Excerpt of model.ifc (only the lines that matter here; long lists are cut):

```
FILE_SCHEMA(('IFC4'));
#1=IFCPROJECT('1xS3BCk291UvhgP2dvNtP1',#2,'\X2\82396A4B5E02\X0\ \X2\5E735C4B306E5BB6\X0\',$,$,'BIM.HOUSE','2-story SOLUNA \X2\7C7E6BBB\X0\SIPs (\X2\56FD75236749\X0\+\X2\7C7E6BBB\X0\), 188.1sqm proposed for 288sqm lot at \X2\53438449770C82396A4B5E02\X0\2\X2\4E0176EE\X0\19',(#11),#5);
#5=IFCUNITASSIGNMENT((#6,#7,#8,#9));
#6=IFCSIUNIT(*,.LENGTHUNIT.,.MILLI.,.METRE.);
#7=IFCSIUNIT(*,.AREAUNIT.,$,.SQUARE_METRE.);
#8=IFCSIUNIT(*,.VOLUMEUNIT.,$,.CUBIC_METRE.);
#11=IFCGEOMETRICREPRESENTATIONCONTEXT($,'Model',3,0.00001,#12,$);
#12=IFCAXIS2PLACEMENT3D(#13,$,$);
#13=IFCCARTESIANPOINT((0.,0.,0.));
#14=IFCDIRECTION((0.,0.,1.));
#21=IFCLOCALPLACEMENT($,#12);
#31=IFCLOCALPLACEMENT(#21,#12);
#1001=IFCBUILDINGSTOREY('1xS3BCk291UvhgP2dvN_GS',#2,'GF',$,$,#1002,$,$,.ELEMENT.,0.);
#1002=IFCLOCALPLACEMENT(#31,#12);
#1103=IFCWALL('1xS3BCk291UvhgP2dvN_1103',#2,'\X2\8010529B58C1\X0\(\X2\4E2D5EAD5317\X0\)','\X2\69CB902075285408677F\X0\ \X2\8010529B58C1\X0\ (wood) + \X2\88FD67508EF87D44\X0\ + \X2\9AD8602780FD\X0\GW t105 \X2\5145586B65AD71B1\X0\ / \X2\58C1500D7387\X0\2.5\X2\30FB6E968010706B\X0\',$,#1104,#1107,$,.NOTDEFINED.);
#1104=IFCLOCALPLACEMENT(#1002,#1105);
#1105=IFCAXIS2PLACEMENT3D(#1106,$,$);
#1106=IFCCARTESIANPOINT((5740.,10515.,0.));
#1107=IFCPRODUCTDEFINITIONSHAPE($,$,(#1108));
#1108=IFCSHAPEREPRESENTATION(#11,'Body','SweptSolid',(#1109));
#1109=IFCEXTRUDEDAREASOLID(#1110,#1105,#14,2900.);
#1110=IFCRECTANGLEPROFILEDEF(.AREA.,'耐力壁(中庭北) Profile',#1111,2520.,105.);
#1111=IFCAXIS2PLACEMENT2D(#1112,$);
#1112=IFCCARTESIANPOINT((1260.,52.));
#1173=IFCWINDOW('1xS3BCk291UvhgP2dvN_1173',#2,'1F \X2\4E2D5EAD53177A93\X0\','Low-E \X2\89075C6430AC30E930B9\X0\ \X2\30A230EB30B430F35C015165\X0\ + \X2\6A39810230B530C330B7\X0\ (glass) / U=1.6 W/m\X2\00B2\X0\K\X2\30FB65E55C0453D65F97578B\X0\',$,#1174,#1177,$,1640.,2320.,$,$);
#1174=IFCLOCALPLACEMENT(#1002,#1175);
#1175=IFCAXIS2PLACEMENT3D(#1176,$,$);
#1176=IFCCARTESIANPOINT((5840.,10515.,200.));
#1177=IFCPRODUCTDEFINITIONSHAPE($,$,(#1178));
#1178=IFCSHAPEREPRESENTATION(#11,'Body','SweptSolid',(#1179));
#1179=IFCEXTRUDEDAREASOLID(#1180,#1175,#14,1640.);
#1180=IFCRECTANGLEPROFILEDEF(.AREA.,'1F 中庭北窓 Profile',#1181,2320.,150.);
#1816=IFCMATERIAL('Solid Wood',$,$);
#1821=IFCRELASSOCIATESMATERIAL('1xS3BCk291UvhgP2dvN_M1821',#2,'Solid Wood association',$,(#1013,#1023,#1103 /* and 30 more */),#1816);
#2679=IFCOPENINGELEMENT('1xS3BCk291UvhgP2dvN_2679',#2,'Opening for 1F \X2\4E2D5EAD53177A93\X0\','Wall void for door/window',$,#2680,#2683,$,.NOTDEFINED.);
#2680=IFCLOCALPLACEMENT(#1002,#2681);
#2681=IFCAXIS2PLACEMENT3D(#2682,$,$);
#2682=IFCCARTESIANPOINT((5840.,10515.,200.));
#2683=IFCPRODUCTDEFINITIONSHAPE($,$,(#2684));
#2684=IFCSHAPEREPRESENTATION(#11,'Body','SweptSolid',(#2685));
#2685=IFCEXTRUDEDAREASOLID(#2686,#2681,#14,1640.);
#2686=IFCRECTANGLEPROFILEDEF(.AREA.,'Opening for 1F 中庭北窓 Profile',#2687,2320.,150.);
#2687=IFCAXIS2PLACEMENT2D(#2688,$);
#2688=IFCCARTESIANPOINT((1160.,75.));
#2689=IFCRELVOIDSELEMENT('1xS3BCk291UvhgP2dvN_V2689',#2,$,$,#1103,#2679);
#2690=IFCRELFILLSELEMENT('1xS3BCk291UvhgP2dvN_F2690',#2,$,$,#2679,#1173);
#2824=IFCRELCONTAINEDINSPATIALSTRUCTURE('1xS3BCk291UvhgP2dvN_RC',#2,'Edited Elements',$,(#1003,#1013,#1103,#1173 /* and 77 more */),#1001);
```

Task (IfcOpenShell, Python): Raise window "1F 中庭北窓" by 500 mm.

```python
import numpy as np
import ifcopenshell
import ifcopenshell.api.geometry
import ifcopenshell.util.placement
import ifcopenshell.util.unit

model = ifcopenshell.open("model.ifc")
unit_scale = ifcopenshell.util.unit.calculate_unit_scale(model)

window = model.by_guid("1xS3BCk291UvhgP2dvN_1173")
opening = window.FillsVoids[0].RelatingOpeningElement
dz = 0.5 / unit_scale

shift = np.array([0.0, 0.0, dz])
# The window is not placed relative to its opening, so move both.
for product in (opening, window):
    matrix = ifcopenshell.util.placement.get_local_placement(product.ObjectPlacement)
    matrix[:3, 3] += shift
    ifcopenshell.api.geometry.edit_object_placement(model, product=product, matrix=matrix, is_si=False)

print(f"moved by {dz * unit_scale:+.3f} m")

model.write("model_updated.ifc")
```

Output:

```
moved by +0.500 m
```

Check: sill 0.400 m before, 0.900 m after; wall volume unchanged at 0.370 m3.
